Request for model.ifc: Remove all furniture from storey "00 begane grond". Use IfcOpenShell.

First a look at what the model holds.

```python
import ifcopenshell
import ifcopenshell.util.element

model = ifcopenshell.open("model.ifc")
print(model.schema)
storey = next(s for s in model.by_type("IfcBuildingStorey") if s.Name == "00 begane grond")
furniture = [e for e in ifcopenshell.util.element.get_decomposition(storey) if e.is_a("IfcFurnishingElement")]
seen = {}
for e in furniture:
    element_type = ifcopenshell.util.element.get_type(e)
    name = element_type.Name if element_type not in (None, e) else None
    seen[name] = seen.get(name, 0) + 1
for name, count in sorted(seen.items(), key=str):
    print(count, "x", name)
```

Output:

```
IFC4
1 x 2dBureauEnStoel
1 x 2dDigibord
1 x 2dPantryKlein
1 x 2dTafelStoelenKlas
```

```python
import ifcopenshell
import ifcopenshell.api.root
import ifcopenshell.util.element

model = ifcopenshell.open("model.ifc")

storey = next(s for s in model.by_type("IfcBuildingStorey") if s.Name == "00 begane grond")
furniture = [e for e in ifcopenshell.util.element.get_decomposition(storey) if e.is_a("IfcFurnishingElement")]

for e in furniture:
    ifcopenshell.api.root.remove_product(model, product=e)
print(len(furniture), "removed")

model.write("model_v2.ifc")
```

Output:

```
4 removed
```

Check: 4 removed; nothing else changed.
